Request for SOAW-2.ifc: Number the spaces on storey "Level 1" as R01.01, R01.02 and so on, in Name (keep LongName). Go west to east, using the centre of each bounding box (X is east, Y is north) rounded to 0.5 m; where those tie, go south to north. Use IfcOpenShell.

First a look at what the model holds.

```python
import ifcopenshell
import ifcopenshell.util.element
import ifcopenshell.util.placement

model = ifcopenshell.open("SOAW-2.ifc")
print(model.schema)
storey = next(s for s in model.by_type("IfcBuildingStorey") if s.Name == "Level 1")
spaces = [e for e in ifcopenshell.util.element.get_decomposition(storey) if e.is_a("IfcSpace")]
for e in sorted(spaces, key=lambda e: e.id()):
    origin = ifcopenshell.util.placement.get_local_placement(e.ObjectPlacement)[:3, 3]
    print(e.id(), e.Name, e.LongName, origin.round(2) + 0.0, sep=" | ")
```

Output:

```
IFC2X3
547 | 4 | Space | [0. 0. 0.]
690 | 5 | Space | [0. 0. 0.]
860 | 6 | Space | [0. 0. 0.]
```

```python
import ifcopenshell
import ifcopenshell.geom
import ifcopenshell.util.element
import ifcopenshell.util.shape

model = ifcopenshell.open("SOAW-2.ifc")
settings = ifcopenshell.geom.settings()
settings.set("use-world-coords", True)


def centre(element):
    shape = ifcopenshell.geom.create_shape(settings, element)
    return ifcopenshell.util.shape.get_bbox_centroid(shape.geometry)


storey = next(s for s in model.by_type("IfcBuildingStorey") if s.Name == "Level 1")
spaces = [e for e in ifcopenshell.util.element.get_decomposition(storey) if e.is_a("IfcSpace")]

# Insertion points can sit at a corner or the storey origin, so sort by the geometry (in metres).
centres = {e: centre(e) for e in spaces}
spaces.sort(key=lambda e: (round(centres[e][0] / 0.5), centres[e][1]))

for i, e in enumerate(spaces, start=1):
    number = f"R01.{i:02d}"
    e.Name = number
    print(e.id(), number)

model.write("SOAW-2_updated.ifc")
```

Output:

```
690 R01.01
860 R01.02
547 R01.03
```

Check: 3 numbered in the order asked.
